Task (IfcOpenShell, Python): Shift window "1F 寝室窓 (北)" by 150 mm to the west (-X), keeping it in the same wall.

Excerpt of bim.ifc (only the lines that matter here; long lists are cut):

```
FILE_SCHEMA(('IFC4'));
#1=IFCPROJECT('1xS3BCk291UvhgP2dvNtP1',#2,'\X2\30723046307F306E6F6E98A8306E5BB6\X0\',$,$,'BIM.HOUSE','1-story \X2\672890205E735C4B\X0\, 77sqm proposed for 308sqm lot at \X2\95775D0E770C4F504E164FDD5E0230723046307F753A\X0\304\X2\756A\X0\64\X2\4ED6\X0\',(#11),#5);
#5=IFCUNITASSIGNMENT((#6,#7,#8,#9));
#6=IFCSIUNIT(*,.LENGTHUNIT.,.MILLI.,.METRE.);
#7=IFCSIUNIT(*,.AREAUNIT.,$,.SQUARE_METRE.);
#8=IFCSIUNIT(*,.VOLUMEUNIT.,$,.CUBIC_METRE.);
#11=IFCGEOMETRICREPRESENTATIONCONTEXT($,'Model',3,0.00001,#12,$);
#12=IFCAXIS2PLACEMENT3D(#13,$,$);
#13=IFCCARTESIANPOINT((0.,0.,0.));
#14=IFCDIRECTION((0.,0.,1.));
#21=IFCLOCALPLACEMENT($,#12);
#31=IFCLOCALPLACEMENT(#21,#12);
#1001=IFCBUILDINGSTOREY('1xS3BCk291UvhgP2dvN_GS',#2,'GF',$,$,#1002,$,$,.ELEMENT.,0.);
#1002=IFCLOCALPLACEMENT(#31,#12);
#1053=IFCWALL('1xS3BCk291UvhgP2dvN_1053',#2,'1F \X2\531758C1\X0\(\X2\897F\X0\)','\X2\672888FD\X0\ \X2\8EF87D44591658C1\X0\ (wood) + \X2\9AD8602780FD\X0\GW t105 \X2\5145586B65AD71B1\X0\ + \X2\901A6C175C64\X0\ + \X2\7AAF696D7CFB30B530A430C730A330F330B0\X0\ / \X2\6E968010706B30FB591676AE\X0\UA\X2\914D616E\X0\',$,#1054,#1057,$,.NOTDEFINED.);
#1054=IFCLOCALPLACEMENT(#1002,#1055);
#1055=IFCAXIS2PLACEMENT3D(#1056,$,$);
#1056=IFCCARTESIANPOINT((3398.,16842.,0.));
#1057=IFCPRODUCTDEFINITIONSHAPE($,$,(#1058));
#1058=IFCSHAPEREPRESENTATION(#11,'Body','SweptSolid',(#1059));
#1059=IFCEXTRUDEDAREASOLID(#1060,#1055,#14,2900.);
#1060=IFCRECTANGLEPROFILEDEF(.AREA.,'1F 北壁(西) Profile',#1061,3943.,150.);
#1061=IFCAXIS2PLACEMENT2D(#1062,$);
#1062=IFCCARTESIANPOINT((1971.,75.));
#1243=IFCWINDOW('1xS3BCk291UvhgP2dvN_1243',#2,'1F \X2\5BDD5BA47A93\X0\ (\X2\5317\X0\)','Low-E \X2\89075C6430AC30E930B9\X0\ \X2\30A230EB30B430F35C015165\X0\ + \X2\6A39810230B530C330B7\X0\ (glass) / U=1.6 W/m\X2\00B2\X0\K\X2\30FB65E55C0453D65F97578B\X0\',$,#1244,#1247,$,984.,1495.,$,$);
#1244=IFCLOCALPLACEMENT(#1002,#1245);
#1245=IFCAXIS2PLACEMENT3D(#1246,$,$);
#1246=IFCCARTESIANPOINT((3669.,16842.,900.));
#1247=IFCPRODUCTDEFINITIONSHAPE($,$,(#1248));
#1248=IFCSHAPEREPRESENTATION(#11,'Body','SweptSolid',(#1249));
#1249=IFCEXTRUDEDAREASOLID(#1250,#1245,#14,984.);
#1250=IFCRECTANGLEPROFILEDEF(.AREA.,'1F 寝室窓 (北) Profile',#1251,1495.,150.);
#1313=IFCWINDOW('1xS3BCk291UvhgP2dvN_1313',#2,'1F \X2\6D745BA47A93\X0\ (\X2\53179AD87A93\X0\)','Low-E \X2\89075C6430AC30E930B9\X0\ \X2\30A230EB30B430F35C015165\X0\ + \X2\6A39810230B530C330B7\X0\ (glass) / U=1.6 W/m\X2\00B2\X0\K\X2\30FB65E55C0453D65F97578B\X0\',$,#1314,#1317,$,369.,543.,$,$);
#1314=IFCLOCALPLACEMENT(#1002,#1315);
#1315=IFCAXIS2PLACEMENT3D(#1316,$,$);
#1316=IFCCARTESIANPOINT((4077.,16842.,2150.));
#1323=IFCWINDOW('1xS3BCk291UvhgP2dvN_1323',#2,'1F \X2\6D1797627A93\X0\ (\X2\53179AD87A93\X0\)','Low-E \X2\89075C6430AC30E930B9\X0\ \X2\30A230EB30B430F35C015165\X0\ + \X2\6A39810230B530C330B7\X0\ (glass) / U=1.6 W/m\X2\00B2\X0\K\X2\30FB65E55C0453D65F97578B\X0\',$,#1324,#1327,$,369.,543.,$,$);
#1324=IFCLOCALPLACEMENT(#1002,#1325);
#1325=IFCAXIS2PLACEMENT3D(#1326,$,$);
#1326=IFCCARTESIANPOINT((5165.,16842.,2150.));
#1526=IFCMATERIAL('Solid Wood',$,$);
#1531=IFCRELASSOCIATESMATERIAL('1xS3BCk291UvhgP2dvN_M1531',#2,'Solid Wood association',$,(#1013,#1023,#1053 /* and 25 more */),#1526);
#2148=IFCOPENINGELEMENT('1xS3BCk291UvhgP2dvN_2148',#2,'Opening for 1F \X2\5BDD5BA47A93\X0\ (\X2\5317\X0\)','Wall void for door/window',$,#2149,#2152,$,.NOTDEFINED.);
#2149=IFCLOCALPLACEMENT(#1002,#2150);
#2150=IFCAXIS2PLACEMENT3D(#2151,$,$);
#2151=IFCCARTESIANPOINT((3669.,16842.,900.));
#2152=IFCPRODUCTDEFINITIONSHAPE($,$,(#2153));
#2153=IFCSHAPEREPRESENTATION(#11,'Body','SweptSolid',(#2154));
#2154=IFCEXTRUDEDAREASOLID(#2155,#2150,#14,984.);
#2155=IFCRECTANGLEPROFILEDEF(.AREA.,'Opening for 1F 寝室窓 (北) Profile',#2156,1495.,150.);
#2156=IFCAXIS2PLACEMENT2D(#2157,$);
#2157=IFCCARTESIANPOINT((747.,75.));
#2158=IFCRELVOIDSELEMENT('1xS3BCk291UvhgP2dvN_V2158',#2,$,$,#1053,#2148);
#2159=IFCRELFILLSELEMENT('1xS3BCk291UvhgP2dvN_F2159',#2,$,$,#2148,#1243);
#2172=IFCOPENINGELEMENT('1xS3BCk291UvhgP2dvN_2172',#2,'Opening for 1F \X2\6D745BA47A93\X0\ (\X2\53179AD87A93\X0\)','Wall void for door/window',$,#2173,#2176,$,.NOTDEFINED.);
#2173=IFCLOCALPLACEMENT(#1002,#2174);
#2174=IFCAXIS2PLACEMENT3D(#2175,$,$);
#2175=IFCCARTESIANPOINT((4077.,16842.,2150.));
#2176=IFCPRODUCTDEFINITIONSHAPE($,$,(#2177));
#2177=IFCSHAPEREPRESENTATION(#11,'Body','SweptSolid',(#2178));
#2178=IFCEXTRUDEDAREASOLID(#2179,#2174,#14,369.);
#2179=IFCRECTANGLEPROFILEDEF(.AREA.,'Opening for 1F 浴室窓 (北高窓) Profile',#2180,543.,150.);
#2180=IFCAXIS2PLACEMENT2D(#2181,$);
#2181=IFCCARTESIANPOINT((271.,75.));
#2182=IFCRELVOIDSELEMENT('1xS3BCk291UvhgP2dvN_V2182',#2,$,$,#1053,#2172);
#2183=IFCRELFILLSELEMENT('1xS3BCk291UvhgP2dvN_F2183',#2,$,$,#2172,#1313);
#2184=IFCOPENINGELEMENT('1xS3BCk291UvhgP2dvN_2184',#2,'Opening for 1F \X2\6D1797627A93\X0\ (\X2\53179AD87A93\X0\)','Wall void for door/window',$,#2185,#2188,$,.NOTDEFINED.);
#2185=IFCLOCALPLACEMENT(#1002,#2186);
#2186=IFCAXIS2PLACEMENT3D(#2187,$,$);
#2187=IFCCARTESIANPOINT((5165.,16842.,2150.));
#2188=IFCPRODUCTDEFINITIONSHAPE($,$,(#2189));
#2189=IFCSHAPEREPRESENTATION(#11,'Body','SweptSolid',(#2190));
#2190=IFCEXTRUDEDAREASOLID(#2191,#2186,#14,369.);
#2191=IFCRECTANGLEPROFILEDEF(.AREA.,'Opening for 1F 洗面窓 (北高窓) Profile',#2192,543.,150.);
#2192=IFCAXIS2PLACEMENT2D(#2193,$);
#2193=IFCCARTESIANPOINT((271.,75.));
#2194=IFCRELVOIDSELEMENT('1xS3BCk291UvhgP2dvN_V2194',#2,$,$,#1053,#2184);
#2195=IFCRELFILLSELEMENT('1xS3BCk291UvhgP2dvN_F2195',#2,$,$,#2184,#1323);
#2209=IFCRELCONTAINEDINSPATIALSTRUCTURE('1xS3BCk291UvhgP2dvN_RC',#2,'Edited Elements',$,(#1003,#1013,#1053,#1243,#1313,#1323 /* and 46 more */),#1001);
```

```python
import ifcopenshell
import ifcopenshell.api.geometry
import ifcopenshell.util.placement

model = ifcopenshell.open("bim.ifc")

window = model.by_guid("1xS3BCk291UvhgP2dvN_1243")
opening = window.FillsVoids[0].RelatingOpeningElement
wall = opening.VoidsElements[0].RelatingBuildingElement

wall_matrix = ifcopenshell.util.placement.get_local_placement(wall.ObjectPlacement)
shift = wall_matrix[:3, 0] * -150.0
before = ifcopenshell.util.placement.get_local_placement(window.ObjectPlacement)[:3, 3].copy()

# The window is not placed relative to its opening, so move both.
for product in (opening, window):
    matrix = ifcopenshell.util.placement.get_local_placement(product.ObjectPlacement)
    matrix[:3, 3] += shift
    ifcopenshell.api.geometry.edit_object_placement(model, product=product, matrix=matrix, is_si=False)

after = ifcopenshell.util.placement.get_local_placement(window.ObjectPlacement)[:3, 3]
print("window moved by", (after - before).round(3) + 0.0)

model.write("bim_v2.ifc")
```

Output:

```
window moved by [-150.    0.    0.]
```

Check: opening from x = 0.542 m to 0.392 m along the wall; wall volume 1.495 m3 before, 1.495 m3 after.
